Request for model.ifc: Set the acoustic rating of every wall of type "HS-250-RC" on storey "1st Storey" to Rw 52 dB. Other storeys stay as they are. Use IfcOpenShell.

First a look at what the model holds.

```python
import ifcopenshell
import ifcopenshell.util.element

model = ifcopenshell.open("model.ifc")
print(model.schema)
storey = next(s for s in model.by_type("IfcBuildingStorey") if s.Name == "1st Storey")
walls = [e for e in ifcopenshell.util.element.get_decomposition(storey) if e.is_a("IfcWall")]
seen = {}
for e in walls:
    element_type = ifcopenshell.util.element.get_type(e)
    key = (element_type.Name if element_type != e and element_type else None, ifcopenshell.util.element.get_pset(e, "Pset_WallCommon", "AcousticRating"))
    seen[key] = seen.get(key, 0) + 1
for (name, value), count in sorted(seen.items(), key=str):
    print(count, "x", name, "|", value)
```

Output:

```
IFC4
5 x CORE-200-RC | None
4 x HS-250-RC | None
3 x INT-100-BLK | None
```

```python
import ifcopenshell
import ifcopenshell.api.pset
import ifcopenshell.util.element

model = ifcopenshell.open("model.ifc")

storey = next(s for s in model.by_type("IfcBuildingStorey") if s.Name == "1st Storey")
walls = [e for e in ifcopenshell.util.element.get_decomposition(storey) if e.is_a("IfcWall")]

count = 0
for e in walls:
    element_type = ifcopenshell.util.element.get_type(e)
    if element_type in (None, e) or element_type.Name != "HS-250-RC":
        continue
    # add_pset returns the element's existing set when there is one.
    pset = ifcopenshell.api.pset.add_pset(model, product=e, name="Pset_WallCommon")
    ifcopenshell.api.pset.edit_pset(model, pset=pset, properties={"AcousticRating": "Rw 52 dB"})
    count += 1

print(count, "walls updated")

model.write("model_v2.ifc")
```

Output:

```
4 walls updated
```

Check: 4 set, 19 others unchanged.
